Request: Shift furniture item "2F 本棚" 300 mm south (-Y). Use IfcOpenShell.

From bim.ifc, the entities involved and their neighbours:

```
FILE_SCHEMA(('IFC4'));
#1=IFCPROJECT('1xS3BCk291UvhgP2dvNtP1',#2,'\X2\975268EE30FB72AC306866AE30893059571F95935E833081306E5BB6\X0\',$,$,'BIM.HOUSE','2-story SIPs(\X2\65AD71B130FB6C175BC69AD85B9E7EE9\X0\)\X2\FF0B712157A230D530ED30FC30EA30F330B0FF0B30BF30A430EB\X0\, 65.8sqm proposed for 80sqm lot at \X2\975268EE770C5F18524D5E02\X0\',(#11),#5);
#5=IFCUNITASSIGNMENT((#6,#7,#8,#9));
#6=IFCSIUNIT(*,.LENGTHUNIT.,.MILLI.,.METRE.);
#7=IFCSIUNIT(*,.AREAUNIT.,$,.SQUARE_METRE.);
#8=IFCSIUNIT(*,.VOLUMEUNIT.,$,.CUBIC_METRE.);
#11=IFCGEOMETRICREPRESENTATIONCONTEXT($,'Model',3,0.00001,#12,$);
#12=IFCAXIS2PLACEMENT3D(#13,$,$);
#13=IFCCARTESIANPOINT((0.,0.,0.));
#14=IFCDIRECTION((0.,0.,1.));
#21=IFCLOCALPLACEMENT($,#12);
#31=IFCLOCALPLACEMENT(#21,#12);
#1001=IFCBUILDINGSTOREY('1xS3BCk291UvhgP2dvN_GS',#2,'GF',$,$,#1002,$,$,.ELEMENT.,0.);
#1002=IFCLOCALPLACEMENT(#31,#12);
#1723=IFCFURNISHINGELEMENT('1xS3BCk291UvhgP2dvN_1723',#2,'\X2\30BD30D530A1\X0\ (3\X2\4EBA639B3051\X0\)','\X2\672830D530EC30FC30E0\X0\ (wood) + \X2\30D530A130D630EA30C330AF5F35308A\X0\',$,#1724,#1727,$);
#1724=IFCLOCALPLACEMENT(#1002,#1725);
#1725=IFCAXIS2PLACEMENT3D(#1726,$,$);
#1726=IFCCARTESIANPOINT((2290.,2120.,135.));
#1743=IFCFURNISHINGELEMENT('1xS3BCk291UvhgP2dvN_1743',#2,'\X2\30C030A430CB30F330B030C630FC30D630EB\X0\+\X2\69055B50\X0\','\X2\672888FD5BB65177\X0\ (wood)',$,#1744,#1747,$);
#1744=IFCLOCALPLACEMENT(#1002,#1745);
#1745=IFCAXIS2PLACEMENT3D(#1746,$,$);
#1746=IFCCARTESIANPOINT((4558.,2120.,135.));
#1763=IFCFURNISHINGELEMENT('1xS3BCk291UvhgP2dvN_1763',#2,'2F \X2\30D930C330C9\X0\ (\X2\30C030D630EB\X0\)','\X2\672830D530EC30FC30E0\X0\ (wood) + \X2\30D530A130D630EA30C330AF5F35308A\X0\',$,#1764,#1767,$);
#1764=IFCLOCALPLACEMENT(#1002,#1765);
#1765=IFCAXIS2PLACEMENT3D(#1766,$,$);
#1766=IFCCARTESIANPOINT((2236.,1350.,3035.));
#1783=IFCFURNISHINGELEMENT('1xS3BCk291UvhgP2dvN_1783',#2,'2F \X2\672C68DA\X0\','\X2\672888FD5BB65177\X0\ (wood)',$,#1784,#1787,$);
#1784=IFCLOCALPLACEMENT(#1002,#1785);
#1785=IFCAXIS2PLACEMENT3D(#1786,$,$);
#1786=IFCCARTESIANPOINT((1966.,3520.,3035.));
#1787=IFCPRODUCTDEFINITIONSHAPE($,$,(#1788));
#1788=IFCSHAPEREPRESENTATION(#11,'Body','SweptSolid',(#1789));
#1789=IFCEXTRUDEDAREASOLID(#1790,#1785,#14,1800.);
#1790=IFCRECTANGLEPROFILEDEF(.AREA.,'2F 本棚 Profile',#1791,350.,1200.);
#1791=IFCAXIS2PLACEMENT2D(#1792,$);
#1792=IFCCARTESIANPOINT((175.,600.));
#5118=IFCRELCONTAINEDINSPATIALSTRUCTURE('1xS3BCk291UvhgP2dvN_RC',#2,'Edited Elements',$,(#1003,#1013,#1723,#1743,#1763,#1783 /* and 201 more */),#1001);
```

```python
import ifcopenshell
import ifcopenshell.api.geometry
import ifcopenshell.util.placement
import ifcopenshell.util.unit

model = ifcopenshell.open("bim.ifc")
unit_scale = ifcopenshell.util.unit.calculate_unit_scale(model)

item = model.by_guid("1xS3BCk291UvhgP2dvN_1783")
matrix = ifcopenshell.util.placement.get_local_placement(item.ObjectPlacement)
matrix[1, 3] -= 0.3 / unit_scale
ifcopenshell.api.geometry.edit_object_placement(model, product=item, matrix=matrix, is_si=False)

print(ifcopenshell.util.placement.get_local_placement(item.ObjectPlacement).round(3) + 0.0)

model.write("bim_edited.ifc")
```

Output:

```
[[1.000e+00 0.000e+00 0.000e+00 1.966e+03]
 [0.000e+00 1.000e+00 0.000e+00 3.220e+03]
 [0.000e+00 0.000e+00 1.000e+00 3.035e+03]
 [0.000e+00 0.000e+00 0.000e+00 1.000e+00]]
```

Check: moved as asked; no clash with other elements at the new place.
